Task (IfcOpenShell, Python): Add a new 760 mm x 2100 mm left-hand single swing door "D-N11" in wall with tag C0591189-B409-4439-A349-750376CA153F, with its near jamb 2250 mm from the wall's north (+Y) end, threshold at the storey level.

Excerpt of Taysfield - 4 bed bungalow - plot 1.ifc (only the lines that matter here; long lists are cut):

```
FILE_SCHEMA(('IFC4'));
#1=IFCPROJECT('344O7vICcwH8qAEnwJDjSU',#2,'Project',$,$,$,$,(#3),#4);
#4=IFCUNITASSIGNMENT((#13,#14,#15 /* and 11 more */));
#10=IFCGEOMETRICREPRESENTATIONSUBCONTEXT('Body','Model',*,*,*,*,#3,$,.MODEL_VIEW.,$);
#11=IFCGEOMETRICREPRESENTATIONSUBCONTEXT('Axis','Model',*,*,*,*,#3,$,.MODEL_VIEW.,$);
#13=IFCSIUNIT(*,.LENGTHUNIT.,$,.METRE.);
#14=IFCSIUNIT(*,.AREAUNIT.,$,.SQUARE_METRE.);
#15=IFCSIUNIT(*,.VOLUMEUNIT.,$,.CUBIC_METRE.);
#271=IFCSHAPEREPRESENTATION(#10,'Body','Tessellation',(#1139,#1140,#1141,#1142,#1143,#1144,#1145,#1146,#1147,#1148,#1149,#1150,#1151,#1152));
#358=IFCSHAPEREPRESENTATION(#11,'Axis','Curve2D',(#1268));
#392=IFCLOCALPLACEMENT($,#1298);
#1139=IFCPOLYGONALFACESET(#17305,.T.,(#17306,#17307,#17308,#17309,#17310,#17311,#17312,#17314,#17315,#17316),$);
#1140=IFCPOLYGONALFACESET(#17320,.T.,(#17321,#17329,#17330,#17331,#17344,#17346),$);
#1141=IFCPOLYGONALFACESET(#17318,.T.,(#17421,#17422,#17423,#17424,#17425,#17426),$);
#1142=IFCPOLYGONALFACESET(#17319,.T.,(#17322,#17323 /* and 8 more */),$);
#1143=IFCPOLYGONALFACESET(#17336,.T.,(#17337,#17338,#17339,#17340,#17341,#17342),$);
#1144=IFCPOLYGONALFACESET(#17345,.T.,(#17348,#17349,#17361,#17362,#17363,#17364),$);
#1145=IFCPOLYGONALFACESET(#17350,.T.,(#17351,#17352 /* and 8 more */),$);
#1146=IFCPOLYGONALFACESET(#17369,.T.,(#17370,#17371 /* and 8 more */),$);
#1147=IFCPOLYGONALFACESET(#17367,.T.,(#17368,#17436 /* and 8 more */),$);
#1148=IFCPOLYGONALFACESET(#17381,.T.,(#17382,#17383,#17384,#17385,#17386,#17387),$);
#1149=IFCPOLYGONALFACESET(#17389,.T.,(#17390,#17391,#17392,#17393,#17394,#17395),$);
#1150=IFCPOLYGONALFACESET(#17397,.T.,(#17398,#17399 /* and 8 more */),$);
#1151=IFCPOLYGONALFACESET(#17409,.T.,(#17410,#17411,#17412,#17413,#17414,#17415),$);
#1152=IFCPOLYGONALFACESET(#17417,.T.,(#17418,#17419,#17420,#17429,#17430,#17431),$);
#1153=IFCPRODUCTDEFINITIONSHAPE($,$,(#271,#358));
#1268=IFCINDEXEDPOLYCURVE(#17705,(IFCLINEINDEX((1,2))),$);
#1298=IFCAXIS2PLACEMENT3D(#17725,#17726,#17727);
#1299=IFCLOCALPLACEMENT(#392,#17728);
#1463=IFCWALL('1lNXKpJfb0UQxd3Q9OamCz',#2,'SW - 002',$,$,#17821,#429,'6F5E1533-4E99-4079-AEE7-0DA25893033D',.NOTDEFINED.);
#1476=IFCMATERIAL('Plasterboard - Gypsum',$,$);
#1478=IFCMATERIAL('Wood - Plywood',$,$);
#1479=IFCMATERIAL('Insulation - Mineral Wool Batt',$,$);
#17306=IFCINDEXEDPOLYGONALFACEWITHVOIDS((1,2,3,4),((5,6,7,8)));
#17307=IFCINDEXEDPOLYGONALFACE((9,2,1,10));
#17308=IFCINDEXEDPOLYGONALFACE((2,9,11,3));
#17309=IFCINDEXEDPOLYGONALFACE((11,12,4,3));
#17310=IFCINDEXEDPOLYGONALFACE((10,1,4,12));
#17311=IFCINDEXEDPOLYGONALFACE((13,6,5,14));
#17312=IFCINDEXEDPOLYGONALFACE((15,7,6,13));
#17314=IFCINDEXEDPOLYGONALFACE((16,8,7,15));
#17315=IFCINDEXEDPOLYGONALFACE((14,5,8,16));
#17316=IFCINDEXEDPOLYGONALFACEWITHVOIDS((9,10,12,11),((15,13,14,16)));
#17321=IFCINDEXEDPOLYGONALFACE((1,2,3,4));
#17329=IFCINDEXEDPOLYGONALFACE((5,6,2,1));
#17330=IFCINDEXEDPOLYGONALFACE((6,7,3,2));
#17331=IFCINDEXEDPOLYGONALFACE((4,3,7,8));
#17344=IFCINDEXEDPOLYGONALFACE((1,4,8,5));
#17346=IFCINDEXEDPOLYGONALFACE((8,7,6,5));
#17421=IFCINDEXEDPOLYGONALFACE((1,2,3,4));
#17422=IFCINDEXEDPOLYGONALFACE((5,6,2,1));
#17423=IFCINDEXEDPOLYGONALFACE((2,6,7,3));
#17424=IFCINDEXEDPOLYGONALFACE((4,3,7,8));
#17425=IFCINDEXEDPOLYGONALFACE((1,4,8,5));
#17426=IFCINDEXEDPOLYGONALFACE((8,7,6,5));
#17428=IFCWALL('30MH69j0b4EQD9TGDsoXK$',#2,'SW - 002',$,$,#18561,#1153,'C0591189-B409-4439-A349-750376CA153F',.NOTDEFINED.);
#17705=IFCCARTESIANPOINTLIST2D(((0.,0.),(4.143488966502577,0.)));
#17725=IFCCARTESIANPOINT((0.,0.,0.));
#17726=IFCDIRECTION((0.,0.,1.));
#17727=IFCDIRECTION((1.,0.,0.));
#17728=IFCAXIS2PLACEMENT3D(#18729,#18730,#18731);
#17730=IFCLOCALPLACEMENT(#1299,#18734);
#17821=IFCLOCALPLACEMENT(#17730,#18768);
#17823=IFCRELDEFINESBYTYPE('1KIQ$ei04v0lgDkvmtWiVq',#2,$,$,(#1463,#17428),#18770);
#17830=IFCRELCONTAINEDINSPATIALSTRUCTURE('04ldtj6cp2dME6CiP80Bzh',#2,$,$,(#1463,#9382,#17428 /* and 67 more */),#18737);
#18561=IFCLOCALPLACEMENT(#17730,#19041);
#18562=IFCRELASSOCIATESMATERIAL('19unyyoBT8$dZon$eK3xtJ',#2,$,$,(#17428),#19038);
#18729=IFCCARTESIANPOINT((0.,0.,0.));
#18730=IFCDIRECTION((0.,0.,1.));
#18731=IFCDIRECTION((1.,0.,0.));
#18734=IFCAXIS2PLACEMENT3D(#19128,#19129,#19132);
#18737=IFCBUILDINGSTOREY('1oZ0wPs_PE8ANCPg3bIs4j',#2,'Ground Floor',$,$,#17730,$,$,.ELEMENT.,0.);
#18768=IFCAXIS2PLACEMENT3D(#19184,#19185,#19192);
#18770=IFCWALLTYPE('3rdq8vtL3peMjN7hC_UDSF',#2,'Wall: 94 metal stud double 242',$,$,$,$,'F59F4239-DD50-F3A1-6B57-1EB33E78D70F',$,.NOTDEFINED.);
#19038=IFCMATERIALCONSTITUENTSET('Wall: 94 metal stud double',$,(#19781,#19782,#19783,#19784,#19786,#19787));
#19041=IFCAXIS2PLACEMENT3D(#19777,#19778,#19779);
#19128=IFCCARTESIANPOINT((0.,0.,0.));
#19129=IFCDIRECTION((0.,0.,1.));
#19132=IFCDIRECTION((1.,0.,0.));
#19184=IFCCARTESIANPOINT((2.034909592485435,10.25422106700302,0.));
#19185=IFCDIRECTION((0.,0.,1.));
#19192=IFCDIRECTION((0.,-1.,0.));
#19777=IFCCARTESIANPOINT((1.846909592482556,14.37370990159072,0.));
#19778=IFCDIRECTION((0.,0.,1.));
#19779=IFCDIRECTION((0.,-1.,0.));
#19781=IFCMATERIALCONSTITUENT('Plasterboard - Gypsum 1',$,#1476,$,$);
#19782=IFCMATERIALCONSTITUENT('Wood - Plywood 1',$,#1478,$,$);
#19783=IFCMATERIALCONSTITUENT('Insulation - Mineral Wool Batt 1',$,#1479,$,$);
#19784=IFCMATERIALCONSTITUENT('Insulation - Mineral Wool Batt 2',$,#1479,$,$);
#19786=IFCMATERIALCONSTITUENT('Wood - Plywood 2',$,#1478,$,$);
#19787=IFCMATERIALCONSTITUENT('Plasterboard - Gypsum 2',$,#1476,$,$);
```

```python
import numpy as np
import ifcopenshell
import ifcopenshell.api.feature
import ifcopenshell.api.geometry
import ifcopenshell.api.root
import ifcopenshell.api.spatial
import ifcopenshell.geom
import ifcopenshell.util.element
import ifcopenshell.util.placement
import ifcopenshell.util.representation
import ifcopenshell.util.shape
import ifcopenshell.util.unit

model = ifcopenshell.open("Taysfield - 4 bed bungalow - plot 1.ifc")
unit_scale = ifcopenshell.util.unit.calculate_unit_scale(model)
settings = ifcopenshell.geom.settings()


def volume(element):
    """Net volume in cubic metres, openings subtracted."""
    shape = ifcopenshell.geom.create_shape(settings, element)
    return ifcopenshell.util.shape.get_volume(shape.geometry)


wall = model.by_guid("30MH69j0b4EQD9TGDsoXK$")
storey = ifcopenshell.util.element.get_container(wall, ifc_class="IfcBuildingStorey")
context = ifcopenshell.util.representation.get_context(model, "Model", "Body", "MODEL_VIEW")
before = volume(wall)

width, height, from_end, sill = 0.76, 2.1, 2.25, 0.0  # metres

# The wall runs along its own X axis, and the end named is its -X end.
wall_shape = ifcopenshell.geom.create_shape(settings, wall)
x, y, z = ifcopenshell.util.shape.get_vertices(wall_shape.geometry).T
start = x.min() + from_end
face, thickness = float(y.min()), float(y.max() - y.min())
wall_matrix = ifcopenshell.util.placement.get_local_placement(wall.ObjectPlacement)
level = ifcopenshell.util.placement.get_local_placement(storey.ObjectPlacement)[2, 3]


def in_wall(x, y):
    """Placement at x, y metres in the wall's axes, at sill height."""
    matrix = wall_matrix.copy()
    matrix[:, 3] = wall_matrix @ np.array([x / unit_scale, y / unit_scale, 0.0, 1.0])
    matrix[2, 3] = level + sill / unit_scale
    return matrix


# Opening: a box that overshoots both wall faces by 50 mm.
opening = ifcopenshell.api.root.create_entity(model, ifc_class="IfcOpeningElement", predefined_type="OPENING")
box = ifcopenshell.api.geometry.add_wall_representation(
    model, context=context, length=width, height=height, thickness=thickness + 0.1
)
ifcopenshell.api.geometry.assign_representation(model, product=opening, representation=box)
ifcopenshell.api.geometry.edit_object_placement(model, product=opening, matrix=in_wall(start, face - 0.05), is_si=False)
ifcopenshell.api.feature.add_feature(model, feature=opening, element=wall)

door = ifcopenshell.api.root.create_entity(model, ifc_class="IfcDoor", name="D-N11", predefined_type="DOOR")
door.OverallWidth, door.OverallHeight = width / unit_scale, height / unit_scale
door.OperationType = "SINGLE_SWING_LEFT"
body = ifcopenshell.api.geometry.add_door_representation(
    model,
    context=context,
    overall_width=door.OverallWidth,
    overall_height=door.OverallHeight,
    operation_type="SINGLE_SWING_LEFT",
    lining_properties={"LiningDepth": thickness / unit_scale, "ThresholdDepth": thickness / unit_scale},
)
ifcopenshell.api.geometry.assign_representation(model, product=door, representation=body)
ifcopenshell.api.spatial.assign_container(model, products=[door], relating_structure=storey)
ifcopenshell.api.feature.add_filling(model, opening=opening, element=door)

# The lining spans the wall, so the door starts at the wall face.
ifcopenshell.api.geometry.edit_object_placement(model, product=door, matrix=in_wall(start, face), is_si=False)

after = volume(wall)

print(f"wall volume {before:.3f} -> {after:.3f} m3")

model.write("Taysfield - 4 bed bungalow - plot 1-out.ifc")
```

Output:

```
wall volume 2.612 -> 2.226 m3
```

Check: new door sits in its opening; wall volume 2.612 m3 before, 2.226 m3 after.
